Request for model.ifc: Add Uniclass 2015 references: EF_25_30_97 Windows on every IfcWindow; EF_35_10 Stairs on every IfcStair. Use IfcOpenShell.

First a look at what the model holds.

```python
import ifcopenshell

model = ifcopenshell.open("model.ifc")
print(model.schema)
print("classifications:", [c.Name for c in model.by_type("IfcClassification")])
for ifc_class in ("IfcDoor", "IfcRoof", "IfcStair", "IfcWall", "IfcWindow"):
    print(ifc_class, len(model.by_type(ifc_class)))
```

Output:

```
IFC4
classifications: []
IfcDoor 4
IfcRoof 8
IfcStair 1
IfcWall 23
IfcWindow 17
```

```python
import ifcopenshell
import ifcopenshell.api.classification

model = ifcopenshell.open("model.ifc")

system = ifcopenshell.api.classification.add_classification(model, classification="Uniclass 2015")

codes = {
    "IfcWindow": ("EF_25_30_97", "Windows"),
    "IfcStair": ("EF_35_10", "Stairs"),
}
for ifc_class, (code, name) in codes.items():
    products = model.by_type(ifc_class)
    ifcopenshell.api.classification.add_reference(
        model, products=products, classification=system, identification=code, name=name
    )
    print(code, len(products))

model.write("model_updated.ifc")
```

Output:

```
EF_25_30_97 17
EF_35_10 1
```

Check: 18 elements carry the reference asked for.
